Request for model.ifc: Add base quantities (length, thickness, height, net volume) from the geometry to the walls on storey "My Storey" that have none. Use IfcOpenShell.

First a look at what the model holds.

```python
import ifcopenshell
import ifcopenshell.util.element
import ifcopenshell.util.unit

model = ifcopenshell.open("model.ifc")
print(model.schema)
for unit_type in ("LENGTHUNIT", "AREAUNIT", "VOLUMEUNIT"):
    print(unit_type, ifcopenshell.util.unit.calculate_unit_scale(model, unit_type))
storey = next(s for s in model.by_type("IfcBuildingStorey") if s.Name == "My Storey")
walls = [e for e in ifcopenshell.util.element.get_decomposition(storey) if e.is_a("IfcWall")]
for e in sorted(walls, key=lambda e: e.id()):
    print(e.id(), e.is_a(), e.Name, list(ifcopenshell.util.element.get_psets(e, qtos_only=True)), sep=" | ")
```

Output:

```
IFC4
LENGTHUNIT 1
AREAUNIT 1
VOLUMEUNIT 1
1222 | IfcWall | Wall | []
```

```python
import ifcopenshell
import ifcopenshell.api.pset
import ifcopenshell.geom
import ifcopenshell.util.element
import ifcopenshell.util.shape
import ifcopenshell.util.unit

model = ifcopenshell.open("model.ifc")
unit_scale = ifcopenshell.util.unit.calculate_unit_scale(model)
volume_scale = ifcopenshell.util.unit.calculate_unit_scale(model, "VOLUMEUNIT")
settings = ifcopenshell.geom.settings()

storey = next(s for s in model.by_type("IfcBuildingStorey") if s.Name == "My Storey")
walls = [e for e in ifcopenshell.util.element.get_decomposition(storey) if e.is_a("IfcWall")]

for e in sorted(walls, key=lambda e: e.id()):
    if ifcopenshell.util.element.get_psets(e, qtos_only=True, should_inherit=False):
        continue
    # Geometry comes back in metres, in the element's own axes.
    shape = ifcopenshell.geom.create_shape(settings, e)
    values = {
        "Length": ifcopenshell.util.shape.get_x(shape.geometry) / unit_scale,
        "Width": ifcopenshell.util.shape.get_y(shape.geometry) / unit_scale,
        "Height": ifcopenshell.util.shape.get_z(shape.geometry) / unit_scale,
        "NetVolume": ifcopenshell.util.shape.get_volume(shape.geometry) / volume_scale,
    }
    qto = ifcopenshell.api.pset.add_qto(model, product=e, name="Qto_WallBaseQuantities")
    ifcopenshell.api.pset.edit_qto(model, qto=qto, properties=values)
    print(e.id(), {k: round(v, 3) for k, v in values.items()})

model.write("model_updated.ifc")
```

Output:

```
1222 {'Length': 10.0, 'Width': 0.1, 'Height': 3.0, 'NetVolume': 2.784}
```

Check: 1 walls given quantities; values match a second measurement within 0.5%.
